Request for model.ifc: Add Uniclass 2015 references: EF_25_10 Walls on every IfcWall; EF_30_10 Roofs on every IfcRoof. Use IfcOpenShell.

First a look at what the model holds.

```python
import ifcopenshell

model = ifcopenshell.open("model.ifc")
print(model.schema)
print("classifications:", [c.Name for c in model.by_type("IfcClassification")])
for ifc_class in ("IfcDoor", "IfcRoof", "IfcStair", "IfcWall", "IfcWindow"):
    print(ifc_class, len(model.by_type(ifc_class)))
```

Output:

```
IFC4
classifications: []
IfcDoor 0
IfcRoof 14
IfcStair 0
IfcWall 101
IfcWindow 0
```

```python
import ifcopenshell
import ifcopenshell.api.classification

model = ifcopenshell.open("model.ifc")

system = ifcopenshell.api.classification.add_classification(model, classification="Uniclass 2015")

codes = {
    "IfcWall": ("EF_25_10", "Walls"),
    "IfcRoof": ("EF_30_10", "Roofs"),
}
for ifc_class, (code, name) in codes.items():
    products = model.by_type(ifc_class)
    ifcopenshell.api.classification.add_reference(
        model, products=products, classification=system, identification=code, name=name
    )
    print(code, len(products))

model.write("model_edited.ifc")
```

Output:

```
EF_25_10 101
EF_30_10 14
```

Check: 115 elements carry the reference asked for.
